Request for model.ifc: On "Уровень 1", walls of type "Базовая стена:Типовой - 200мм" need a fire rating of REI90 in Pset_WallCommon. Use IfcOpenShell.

First a look at what the model holds.

```python
import ifcopenshell
import ifcopenshell.util.element

model = ifcopenshell.open("model.ifc")
print(model.schema)
storey = next(s for s in model.by_type("IfcBuildingStorey") if s.Name == "Уровень 1")
walls = [e for e in ifcopenshell.util.element.get_decomposition(storey) if e.is_a("IfcWall")]
seen = {}
for e in walls:
    element_type = ifcopenshell.util.element.get_type(e)
    key = (element_type.Name if element_type != e and element_type else None, ifcopenshell.util.element.get_pset(e, "Pset_WallCommon", "FireRating"))
    seen[key] = seen.get(key, 0) + 1
for (name, value), count in sorted(seen.items(), key=str):
    print(count, "x", name, "|", value)
```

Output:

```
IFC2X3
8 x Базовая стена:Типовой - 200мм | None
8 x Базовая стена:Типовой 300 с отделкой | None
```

```python
import ifcopenshell
import ifcopenshell.api.pset
import ifcopenshell.util.element

model = ifcopenshell.open("model.ifc")

storey = next(s for s in model.by_type("IfcBuildingStorey") if s.Name == "Уровень 1")
walls = [e for e in ifcopenshell.util.element.get_decomposition(storey) if e.is_a("IfcWall")]

count = 0
for e in walls:
    element_type = ifcopenshell.util.element.get_type(e)
    if element_type in (None, e) or element_type.Name != "Базовая стена:Типовой - 200мм":
        continue
    # add_pset returns the element's existing set when there is one.
    pset = ifcopenshell.api.pset.add_pset(model, product=e, name="Pset_WallCommon")
    ifcopenshell.api.pset.edit_pset(model, pset=pset, properties={"FireRating": "REI90"})
    count += 1

print(count, "walls updated")

model.write("model_edited.ifc")
```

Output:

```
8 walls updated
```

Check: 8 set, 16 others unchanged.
